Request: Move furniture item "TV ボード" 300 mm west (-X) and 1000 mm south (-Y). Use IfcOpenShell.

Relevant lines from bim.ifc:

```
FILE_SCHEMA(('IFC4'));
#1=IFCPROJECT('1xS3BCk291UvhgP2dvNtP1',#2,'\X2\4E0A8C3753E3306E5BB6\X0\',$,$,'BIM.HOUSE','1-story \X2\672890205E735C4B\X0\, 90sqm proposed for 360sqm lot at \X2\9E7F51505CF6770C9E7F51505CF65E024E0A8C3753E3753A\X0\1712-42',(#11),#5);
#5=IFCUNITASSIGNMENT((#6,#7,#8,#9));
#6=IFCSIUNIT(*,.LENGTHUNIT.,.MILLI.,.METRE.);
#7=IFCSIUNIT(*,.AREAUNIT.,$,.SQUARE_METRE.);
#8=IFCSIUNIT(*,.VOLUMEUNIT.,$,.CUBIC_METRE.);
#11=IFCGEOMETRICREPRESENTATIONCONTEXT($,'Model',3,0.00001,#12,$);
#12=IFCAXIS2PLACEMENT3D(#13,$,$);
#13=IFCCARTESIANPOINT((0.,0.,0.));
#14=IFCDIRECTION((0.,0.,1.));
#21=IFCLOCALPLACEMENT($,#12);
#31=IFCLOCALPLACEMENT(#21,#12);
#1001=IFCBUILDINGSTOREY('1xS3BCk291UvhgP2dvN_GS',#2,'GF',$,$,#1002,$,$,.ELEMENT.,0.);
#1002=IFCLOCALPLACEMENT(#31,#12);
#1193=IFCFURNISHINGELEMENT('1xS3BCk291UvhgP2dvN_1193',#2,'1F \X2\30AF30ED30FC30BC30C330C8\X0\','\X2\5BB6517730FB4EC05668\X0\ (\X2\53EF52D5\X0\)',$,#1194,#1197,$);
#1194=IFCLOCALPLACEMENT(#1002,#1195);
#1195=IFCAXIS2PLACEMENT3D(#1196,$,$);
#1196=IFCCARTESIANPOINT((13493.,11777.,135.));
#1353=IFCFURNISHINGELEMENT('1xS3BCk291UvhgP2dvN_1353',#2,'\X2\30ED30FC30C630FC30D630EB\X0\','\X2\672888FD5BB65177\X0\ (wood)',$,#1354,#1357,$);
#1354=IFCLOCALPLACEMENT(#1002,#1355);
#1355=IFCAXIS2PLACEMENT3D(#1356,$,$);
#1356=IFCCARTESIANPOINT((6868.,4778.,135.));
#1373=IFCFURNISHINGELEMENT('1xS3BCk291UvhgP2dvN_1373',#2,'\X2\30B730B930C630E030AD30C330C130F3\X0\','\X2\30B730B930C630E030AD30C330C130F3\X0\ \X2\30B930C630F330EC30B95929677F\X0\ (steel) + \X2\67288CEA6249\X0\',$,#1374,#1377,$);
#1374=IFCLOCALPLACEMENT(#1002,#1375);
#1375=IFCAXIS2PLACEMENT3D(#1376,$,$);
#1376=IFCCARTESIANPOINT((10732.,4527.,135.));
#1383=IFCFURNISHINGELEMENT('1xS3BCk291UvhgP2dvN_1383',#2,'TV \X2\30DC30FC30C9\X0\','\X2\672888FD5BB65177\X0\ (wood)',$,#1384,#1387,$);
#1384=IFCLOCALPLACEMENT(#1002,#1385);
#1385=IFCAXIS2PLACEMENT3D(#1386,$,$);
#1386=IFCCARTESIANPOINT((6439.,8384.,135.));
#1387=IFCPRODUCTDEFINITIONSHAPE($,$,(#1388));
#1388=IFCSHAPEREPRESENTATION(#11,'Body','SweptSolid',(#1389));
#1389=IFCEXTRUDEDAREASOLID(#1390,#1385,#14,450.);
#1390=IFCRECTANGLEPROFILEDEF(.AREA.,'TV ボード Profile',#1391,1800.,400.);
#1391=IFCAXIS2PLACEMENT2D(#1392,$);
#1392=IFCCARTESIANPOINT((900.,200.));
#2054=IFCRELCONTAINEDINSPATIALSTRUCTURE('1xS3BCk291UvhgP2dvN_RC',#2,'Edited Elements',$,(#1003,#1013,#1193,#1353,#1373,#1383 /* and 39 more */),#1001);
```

```python
import ifcopenshell
import ifcopenshell.api.geometry
import ifcopenshell.util.placement
import ifcopenshell.util.unit

model = ifcopenshell.open("bim.ifc")
unit_scale = ifcopenshell.util.unit.calculate_unit_scale(model)

item = model.by_id(1383)
matrix = ifcopenshell.util.placement.get_local_placement(item.ObjectPlacement)
matrix[0, 3] -= 0.3 / unit_scale
matrix[1, 3] -= 1 / unit_scale
ifcopenshell.api.geometry.edit_object_placement(model, product=item, matrix=matrix, is_si=False)

print(ifcopenshell.util.placement.get_local_placement(item.ObjectPlacement).round(3) + 0.0)

model.write("bim_v2.ifc")
```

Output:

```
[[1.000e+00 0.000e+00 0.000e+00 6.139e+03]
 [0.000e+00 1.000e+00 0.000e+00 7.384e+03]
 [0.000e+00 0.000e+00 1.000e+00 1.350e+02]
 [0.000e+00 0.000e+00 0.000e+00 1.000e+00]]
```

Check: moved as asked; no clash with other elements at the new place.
